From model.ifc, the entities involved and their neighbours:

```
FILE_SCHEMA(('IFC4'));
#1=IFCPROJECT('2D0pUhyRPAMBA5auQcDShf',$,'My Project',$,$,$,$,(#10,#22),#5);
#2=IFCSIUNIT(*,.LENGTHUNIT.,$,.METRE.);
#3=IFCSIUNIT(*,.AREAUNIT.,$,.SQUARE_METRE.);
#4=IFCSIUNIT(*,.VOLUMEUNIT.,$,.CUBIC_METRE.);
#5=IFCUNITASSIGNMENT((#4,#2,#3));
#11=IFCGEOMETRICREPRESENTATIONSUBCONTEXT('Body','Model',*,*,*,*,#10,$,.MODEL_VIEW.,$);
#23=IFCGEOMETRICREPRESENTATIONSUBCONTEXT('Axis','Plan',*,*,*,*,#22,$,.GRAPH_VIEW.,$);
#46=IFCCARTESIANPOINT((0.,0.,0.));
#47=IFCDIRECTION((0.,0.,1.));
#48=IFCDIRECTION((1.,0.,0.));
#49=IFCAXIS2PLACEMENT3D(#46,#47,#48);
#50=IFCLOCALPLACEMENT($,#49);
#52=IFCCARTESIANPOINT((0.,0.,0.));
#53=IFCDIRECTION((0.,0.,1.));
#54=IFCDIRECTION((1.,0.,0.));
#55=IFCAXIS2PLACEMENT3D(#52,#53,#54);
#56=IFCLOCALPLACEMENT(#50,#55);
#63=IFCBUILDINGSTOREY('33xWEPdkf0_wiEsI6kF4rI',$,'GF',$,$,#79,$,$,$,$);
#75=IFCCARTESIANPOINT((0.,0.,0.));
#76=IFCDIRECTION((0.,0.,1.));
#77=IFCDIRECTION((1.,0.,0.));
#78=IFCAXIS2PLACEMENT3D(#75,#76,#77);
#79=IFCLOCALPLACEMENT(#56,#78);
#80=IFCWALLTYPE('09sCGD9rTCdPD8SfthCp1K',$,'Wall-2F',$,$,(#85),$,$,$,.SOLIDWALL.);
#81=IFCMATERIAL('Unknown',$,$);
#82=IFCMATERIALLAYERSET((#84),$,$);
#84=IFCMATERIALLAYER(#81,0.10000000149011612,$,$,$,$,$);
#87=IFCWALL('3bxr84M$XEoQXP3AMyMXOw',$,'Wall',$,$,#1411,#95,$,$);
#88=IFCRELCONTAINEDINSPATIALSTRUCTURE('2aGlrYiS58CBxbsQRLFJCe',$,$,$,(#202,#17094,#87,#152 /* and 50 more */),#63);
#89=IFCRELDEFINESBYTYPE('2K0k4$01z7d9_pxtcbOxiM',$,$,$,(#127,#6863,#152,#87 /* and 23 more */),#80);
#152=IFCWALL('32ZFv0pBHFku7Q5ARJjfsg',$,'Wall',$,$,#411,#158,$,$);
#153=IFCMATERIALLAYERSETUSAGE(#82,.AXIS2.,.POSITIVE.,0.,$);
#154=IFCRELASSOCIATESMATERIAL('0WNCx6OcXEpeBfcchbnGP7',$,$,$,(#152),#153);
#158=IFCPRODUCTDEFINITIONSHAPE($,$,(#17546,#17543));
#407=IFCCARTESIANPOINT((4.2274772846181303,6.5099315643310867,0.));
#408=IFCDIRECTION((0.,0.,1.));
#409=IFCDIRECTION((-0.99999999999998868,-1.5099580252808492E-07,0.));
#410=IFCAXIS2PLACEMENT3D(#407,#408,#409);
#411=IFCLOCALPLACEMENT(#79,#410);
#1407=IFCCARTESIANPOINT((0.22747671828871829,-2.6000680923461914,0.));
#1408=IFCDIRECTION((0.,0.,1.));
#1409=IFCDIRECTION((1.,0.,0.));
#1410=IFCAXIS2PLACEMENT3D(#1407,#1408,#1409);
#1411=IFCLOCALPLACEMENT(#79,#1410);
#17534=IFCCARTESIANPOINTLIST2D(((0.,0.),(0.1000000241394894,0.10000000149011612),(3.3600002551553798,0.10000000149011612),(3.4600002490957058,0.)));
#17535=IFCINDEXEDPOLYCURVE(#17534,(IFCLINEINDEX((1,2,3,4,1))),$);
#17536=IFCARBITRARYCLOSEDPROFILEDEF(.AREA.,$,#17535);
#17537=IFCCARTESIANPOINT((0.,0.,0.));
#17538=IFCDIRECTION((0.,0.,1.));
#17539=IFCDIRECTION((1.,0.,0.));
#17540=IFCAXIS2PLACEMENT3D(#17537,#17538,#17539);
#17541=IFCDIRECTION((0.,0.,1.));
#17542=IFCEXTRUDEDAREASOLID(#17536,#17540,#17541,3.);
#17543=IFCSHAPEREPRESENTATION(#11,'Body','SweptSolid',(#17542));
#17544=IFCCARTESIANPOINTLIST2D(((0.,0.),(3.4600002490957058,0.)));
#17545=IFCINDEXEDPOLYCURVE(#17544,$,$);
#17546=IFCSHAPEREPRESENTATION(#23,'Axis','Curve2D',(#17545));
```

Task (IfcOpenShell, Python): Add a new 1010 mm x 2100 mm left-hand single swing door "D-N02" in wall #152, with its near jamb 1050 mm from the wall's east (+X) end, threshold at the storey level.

```python
import numpy as np
import ifcopenshell
import ifcopenshell.api.feature
import ifcopenshell.api.geometry
import ifcopenshell.api.root
import ifcopenshell.api.spatial
import ifcopenshell.geom
import ifcopenshell.util.element
import ifcopenshell.util.placement
import ifcopenshell.util.representation
import ifcopenshell.util.shape
import ifcopenshell.util.unit

model = ifcopenshell.open("model.ifc")
unit_scale = ifcopenshell.util.unit.calculate_unit_scale(model)
settings = ifcopenshell.geom.settings()


def volume(element):
    """Net volume in cubic metres, openings subtracted."""
    shape = ifcopenshell.geom.create_shape(settings, element)
    return ifcopenshell.util.shape.get_volume(shape.geometry)


wall = model.by_guid("32ZFv0pBHFku7Q5ARJjfsg")
storey = ifcopenshell.util.element.get_container(wall, ifc_class="IfcBuildingStorey")
context = ifcopenshell.util.representation.get_context(model, "Model", "Body", "MODEL_VIEW")
before = volume(wall)

width, height, from_end, sill = 1.01, 2.1, 1.05, 0.0  # metres

# The wall runs along its own X axis, and the end named is its -X end.
wall_shape = ifcopenshell.geom.create_shape(settings, wall)
x, y, z = ifcopenshell.util.shape.get_vertices(wall_shape.geometry).T
start = x.min() + from_end
face, thickness = float(y.min()), float(y.max() - y.min())
wall_matrix = ifcopenshell.util.placement.get_local_placement(wall.ObjectPlacement)
level = ifcopenshell.util.placement.get_local_placement(storey.ObjectPlacement)[2, 3]


def in_wall(x, y):
    """Placement at x, y metres in the wall's axes, at sill height."""
    matrix = wall_matrix.copy()
    matrix[:, 3] = wall_matrix @ np.array([x / unit_scale, y / unit_scale, 0.0, 1.0])
    matrix[2, 3] = level + sill / unit_scale
    return matrix


# Opening: a box that overshoots both wall faces by 50 mm.
opening = ifcopenshell.api.root.create_entity(model, ifc_class="IfcOpeningElement", predefined_type="OPENING")
box = ifcopenshell.api.geometry.add_wall_representation(
    model, context=context, length=width, height=height, thickness=thickness + 0.1
)
ifcopenshell.api.geometry.assign_representation(model, product=opening, representation=box)
ifcopenshell.api.geometry.edit_object_placement(model, product=opening, matrix=in_wall(start, face - 0.05), is_si=False)
ifcopenshell.api.feature.add_feature(model, feature=opening, element=wall)

door = ifcopenshell.api.root.create_entity(model, ifc_class="IfcDoor", name="D-N02", predefined_type="DOOR")
door.OverallWidth, door.OverallHeight = width / unit_scale, height / unit_scale
door.OperationType = "SINGLE_SWING_LEFT"
body = ifcopenshell.api.geometry.add_door_representation(
    model,
    context=context,
    overall_width=door.OverallWidth,
    overall_height=door.OverallHeight,
    operation_type="SINGLE_SWING_LEFT",
    lining_properties={"LiningDepth": thickness / unit_scale, "ThresholdDepth": thickness / unit_scale},
)
ifcopenshell.api.geometry.assign_representation(model, product=door, representation=body)
ifcopenshell.api.spatial.assign_container(model, products=[door], relating_structure=storey)
ifcopenshell.api.feature.add_filling(model, opening=opening, element=door)

# The lining spans the wall, so the door starts at the wall face.
ifcopenshell.api.geometry.edit_object_placement(model, product=door, matrix=in_wall(start, face), is_si=False)

after = volume(wall)

print(f"wall volume {before:.3f} -> {after:.3f} m3")

model.write("model_edited.ifc")
```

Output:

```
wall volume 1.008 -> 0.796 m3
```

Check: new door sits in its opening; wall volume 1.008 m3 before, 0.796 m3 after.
